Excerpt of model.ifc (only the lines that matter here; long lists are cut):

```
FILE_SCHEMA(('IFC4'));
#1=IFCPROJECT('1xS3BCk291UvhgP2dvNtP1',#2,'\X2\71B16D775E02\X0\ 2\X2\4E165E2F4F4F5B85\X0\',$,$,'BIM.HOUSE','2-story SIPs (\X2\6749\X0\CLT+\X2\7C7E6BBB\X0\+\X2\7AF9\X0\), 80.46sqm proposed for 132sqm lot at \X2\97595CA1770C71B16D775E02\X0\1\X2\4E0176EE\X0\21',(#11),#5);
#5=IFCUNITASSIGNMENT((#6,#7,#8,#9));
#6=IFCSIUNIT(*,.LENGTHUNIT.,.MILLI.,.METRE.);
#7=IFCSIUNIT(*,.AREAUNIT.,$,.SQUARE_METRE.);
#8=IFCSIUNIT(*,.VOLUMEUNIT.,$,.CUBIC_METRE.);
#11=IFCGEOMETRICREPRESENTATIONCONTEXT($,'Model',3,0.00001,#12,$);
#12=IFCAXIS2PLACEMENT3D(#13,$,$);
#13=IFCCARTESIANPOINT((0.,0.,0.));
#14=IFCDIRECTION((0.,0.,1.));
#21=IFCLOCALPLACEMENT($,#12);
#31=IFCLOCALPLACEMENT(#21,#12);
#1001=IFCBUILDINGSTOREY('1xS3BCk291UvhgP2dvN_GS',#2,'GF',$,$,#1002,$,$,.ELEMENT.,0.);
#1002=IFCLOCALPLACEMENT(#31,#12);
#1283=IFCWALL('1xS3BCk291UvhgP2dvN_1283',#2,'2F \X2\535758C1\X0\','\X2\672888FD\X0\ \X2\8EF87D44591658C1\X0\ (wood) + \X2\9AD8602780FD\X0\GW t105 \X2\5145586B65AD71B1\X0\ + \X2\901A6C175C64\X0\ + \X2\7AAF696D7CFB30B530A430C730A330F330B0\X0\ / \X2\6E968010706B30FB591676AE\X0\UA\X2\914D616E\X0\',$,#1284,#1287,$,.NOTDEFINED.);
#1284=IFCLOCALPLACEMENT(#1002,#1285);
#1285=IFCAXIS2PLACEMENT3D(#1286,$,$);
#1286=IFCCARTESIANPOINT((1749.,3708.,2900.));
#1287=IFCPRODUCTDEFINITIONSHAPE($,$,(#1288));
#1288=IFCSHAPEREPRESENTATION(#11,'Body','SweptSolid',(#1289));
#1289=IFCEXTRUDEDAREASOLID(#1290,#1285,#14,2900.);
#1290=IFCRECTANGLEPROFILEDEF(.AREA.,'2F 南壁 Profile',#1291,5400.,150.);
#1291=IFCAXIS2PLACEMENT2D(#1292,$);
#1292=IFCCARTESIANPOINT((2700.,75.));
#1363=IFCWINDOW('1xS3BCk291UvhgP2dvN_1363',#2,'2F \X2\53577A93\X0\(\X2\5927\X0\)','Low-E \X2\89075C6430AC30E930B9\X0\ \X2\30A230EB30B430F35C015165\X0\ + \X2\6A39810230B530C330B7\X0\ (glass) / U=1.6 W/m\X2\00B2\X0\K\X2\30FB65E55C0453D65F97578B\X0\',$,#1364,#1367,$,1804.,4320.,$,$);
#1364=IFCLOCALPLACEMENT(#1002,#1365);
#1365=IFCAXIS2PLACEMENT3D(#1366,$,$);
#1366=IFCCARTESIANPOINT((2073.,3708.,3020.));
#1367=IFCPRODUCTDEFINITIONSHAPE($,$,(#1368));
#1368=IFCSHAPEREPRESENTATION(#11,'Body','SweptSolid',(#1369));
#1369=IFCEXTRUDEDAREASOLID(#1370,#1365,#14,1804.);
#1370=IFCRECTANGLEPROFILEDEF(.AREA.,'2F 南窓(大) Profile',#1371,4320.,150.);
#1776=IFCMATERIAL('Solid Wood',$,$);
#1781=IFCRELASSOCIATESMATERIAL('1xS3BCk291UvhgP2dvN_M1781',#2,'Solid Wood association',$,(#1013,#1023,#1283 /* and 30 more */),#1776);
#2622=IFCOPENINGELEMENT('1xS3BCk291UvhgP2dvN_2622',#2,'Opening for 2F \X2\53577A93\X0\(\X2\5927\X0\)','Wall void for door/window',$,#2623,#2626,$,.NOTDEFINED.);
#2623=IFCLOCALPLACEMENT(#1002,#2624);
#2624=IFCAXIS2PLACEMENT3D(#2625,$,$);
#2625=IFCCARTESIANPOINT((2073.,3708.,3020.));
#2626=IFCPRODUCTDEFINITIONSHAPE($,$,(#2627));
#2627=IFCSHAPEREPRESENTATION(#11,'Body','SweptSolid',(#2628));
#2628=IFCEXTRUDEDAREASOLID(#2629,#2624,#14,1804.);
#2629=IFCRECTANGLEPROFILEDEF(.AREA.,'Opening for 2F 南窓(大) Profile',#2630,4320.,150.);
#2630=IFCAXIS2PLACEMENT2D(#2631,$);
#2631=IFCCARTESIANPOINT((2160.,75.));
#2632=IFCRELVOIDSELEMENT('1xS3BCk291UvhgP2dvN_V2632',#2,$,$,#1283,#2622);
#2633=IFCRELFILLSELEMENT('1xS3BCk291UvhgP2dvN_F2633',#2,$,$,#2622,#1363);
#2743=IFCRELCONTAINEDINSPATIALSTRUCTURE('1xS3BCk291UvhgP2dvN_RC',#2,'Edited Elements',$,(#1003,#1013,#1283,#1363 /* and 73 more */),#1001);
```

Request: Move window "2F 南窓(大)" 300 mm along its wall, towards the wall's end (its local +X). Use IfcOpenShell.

```python
import ifcopenshell
import ifcopenshell.api.geometry
import ifcopenshell.util.placement
import ifcopenshell.util.unit

model = ifcopenshell.open("model.ifc")
unit_scale = ifcopenshell.util.unit.calculate_unit_scale(model)

window = model.by_guid("1xS3BCk291UvhgP2dvN_1363")
opening = window.FillsVoids[0].RelatingOpeningElement
wall = opening.VoidsElements[0].RelatingBuildingElement

wall_matrix = ifcopenshell.util.placement.get_local_placement(wall.ObjectPlacement)
shift = wall_matrix[:3, 0] * 0.3 / unit_scale
before = ifcopenshell.util.placement.get_local_placement(window.ObjectPlacement)[:3, 3].copy()

# The window is not placed relative to its opening, so move both.
for product in (opening, window):
    matrix = ifcopenshell.util.placement.get_local_placement(product.ObjectPlacement)
    matrix[:3, 3] += shift
    ifcopenshell.api.geometry.edit_object_placement(model, product=product, matrix=matrix, is_si=False)

after = ifcopenshell.util.placement.get_local_placement(window.ObjectPlacement)[:3, 3]
print("window moved by", (after - before).round(3) + 0.0)

model.write("model_updated.ifc")
```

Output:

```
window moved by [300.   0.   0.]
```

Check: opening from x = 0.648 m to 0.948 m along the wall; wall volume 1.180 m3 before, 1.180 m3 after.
